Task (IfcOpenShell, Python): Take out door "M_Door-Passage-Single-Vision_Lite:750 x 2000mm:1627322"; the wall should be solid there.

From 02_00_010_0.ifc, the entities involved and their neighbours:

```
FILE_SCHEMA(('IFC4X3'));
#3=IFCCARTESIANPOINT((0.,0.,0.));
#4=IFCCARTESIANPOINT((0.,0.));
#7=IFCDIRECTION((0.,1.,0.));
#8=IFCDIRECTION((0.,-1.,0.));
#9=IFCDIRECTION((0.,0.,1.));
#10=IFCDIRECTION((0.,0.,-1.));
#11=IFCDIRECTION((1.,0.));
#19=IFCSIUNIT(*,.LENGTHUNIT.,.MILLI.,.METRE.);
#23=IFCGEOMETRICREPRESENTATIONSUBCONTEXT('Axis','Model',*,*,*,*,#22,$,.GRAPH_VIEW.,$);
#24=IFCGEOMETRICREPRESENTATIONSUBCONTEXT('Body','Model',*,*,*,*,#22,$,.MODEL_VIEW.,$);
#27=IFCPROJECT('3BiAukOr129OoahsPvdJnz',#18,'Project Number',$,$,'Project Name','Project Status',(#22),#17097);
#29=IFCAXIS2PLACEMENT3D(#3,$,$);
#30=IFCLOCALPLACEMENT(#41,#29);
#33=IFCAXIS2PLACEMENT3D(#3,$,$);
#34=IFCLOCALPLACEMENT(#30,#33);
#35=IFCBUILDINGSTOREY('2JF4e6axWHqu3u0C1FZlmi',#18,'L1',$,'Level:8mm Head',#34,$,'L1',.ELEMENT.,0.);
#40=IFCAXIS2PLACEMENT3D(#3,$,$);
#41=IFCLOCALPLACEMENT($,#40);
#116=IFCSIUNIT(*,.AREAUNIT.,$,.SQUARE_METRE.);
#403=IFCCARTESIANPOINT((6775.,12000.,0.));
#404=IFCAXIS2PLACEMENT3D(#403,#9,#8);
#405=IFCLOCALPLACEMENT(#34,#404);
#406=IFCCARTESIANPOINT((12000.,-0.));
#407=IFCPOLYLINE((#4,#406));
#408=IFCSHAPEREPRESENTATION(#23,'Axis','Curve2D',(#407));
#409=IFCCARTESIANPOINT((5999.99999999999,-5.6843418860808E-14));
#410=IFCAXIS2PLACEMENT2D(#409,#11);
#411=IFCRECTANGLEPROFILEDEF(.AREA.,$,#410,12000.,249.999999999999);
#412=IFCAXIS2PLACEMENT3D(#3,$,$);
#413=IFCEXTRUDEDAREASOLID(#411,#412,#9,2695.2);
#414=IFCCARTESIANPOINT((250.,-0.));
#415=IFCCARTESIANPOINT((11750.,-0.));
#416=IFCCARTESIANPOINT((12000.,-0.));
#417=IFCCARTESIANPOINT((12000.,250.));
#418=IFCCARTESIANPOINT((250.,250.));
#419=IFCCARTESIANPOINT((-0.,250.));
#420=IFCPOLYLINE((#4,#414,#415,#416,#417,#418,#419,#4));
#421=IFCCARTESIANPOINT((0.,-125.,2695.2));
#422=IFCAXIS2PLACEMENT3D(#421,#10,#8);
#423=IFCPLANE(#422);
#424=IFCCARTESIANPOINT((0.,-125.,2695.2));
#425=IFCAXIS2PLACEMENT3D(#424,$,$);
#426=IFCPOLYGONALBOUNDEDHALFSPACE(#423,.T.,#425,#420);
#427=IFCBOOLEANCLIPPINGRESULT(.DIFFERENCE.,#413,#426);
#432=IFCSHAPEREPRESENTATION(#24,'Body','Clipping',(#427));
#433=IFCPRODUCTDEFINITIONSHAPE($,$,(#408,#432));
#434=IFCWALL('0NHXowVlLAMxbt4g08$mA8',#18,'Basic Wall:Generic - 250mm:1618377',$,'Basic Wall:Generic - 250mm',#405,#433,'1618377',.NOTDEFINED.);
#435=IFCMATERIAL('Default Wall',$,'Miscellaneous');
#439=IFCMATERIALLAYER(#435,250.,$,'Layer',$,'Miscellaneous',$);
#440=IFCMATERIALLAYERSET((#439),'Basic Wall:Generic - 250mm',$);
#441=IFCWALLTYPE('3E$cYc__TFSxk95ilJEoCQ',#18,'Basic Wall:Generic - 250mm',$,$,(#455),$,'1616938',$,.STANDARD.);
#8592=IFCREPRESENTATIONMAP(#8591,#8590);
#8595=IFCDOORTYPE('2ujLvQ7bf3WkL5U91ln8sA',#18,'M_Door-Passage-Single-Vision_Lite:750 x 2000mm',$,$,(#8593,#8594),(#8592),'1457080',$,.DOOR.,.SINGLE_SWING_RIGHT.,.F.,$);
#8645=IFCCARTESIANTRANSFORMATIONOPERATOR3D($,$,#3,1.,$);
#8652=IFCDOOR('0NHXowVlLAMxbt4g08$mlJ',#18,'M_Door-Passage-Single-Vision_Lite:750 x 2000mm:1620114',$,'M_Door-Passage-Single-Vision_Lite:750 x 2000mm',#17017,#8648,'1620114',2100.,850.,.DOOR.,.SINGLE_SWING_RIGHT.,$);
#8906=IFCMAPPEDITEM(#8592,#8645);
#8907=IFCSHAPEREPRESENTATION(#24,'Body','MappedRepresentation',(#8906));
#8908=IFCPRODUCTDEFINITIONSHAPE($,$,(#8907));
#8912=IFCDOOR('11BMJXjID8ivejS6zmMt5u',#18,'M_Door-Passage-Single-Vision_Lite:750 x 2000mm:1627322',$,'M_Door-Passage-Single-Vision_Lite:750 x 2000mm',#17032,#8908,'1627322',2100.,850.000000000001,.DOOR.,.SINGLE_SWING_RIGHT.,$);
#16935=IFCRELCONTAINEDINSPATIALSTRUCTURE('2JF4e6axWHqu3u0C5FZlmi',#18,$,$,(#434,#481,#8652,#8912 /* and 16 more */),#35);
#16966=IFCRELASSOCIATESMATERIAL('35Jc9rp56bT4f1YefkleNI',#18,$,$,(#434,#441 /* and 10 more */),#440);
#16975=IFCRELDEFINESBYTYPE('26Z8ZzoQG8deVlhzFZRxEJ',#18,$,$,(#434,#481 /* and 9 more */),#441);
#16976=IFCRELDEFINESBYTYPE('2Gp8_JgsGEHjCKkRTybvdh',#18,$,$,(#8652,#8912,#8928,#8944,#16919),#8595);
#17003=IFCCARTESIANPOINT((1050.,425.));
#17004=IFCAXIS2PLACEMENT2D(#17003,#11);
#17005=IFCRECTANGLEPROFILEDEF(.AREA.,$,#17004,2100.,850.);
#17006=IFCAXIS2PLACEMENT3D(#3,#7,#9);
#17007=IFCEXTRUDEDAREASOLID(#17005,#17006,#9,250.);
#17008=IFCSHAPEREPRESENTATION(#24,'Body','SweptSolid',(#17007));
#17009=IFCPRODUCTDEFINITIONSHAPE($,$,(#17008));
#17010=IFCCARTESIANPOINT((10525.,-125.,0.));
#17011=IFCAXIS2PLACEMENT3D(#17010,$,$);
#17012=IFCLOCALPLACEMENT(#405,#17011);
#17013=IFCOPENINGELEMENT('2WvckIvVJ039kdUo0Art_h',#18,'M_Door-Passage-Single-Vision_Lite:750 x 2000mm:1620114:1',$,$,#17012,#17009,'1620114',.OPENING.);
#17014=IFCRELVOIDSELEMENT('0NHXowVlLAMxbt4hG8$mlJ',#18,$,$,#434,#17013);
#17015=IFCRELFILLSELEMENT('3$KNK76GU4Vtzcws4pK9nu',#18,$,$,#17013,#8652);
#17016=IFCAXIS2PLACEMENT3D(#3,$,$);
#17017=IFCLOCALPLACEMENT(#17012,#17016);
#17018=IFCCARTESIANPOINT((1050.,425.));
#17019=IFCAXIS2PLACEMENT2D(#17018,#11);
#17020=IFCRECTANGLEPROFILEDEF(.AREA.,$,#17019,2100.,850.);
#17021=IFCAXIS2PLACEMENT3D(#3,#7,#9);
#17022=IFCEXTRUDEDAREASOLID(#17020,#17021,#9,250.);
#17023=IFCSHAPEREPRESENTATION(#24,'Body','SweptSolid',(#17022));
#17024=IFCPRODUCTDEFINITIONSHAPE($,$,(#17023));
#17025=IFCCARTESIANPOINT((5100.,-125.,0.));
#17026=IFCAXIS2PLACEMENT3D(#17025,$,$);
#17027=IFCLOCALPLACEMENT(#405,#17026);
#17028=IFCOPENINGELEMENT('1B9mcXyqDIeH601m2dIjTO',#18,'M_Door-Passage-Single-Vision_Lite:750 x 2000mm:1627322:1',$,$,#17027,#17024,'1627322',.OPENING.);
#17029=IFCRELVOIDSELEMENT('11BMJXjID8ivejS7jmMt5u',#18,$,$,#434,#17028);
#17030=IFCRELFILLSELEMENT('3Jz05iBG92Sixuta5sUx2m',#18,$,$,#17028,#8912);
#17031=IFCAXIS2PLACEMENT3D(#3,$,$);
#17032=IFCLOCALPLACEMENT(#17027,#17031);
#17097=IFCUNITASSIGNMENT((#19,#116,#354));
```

```python
import ifcopenshell
import ifcopenshell.api.feature
import ifcopenshell.api.root
import ifcopenshell.geom
import ifcopenshell.util.shape

model = ifcopenshell.open("02_00_010_0.ifc")
settings = ifcopenshell.geom.settings()


def volume(element):
    """Net volume in cubic metres, openings subtracted."""
    shape = ifcopenshell.geom.create_shape(settings, element)
    return ifcopenshell.util.shape.get_volume(shape.geometry)


door = model.by_id(8912)
opening = door.FillsVoids[0].RelatingOpeningElement
wall = opening.VoidsElements[0].RelatingBuildingElement
before = volume(wall)

ifcopenshell.api.root.remove_product(model, product=door)
ifcopenshell.api.feature.remove_feature(model, feature=opening)

after = volume(wall)

print(f"wall volume {before:.3f} -> {after:.3f} m3")

model.write("02_00_010_0_rev.ifc")
```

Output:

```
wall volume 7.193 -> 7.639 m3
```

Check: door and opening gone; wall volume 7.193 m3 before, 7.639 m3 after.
